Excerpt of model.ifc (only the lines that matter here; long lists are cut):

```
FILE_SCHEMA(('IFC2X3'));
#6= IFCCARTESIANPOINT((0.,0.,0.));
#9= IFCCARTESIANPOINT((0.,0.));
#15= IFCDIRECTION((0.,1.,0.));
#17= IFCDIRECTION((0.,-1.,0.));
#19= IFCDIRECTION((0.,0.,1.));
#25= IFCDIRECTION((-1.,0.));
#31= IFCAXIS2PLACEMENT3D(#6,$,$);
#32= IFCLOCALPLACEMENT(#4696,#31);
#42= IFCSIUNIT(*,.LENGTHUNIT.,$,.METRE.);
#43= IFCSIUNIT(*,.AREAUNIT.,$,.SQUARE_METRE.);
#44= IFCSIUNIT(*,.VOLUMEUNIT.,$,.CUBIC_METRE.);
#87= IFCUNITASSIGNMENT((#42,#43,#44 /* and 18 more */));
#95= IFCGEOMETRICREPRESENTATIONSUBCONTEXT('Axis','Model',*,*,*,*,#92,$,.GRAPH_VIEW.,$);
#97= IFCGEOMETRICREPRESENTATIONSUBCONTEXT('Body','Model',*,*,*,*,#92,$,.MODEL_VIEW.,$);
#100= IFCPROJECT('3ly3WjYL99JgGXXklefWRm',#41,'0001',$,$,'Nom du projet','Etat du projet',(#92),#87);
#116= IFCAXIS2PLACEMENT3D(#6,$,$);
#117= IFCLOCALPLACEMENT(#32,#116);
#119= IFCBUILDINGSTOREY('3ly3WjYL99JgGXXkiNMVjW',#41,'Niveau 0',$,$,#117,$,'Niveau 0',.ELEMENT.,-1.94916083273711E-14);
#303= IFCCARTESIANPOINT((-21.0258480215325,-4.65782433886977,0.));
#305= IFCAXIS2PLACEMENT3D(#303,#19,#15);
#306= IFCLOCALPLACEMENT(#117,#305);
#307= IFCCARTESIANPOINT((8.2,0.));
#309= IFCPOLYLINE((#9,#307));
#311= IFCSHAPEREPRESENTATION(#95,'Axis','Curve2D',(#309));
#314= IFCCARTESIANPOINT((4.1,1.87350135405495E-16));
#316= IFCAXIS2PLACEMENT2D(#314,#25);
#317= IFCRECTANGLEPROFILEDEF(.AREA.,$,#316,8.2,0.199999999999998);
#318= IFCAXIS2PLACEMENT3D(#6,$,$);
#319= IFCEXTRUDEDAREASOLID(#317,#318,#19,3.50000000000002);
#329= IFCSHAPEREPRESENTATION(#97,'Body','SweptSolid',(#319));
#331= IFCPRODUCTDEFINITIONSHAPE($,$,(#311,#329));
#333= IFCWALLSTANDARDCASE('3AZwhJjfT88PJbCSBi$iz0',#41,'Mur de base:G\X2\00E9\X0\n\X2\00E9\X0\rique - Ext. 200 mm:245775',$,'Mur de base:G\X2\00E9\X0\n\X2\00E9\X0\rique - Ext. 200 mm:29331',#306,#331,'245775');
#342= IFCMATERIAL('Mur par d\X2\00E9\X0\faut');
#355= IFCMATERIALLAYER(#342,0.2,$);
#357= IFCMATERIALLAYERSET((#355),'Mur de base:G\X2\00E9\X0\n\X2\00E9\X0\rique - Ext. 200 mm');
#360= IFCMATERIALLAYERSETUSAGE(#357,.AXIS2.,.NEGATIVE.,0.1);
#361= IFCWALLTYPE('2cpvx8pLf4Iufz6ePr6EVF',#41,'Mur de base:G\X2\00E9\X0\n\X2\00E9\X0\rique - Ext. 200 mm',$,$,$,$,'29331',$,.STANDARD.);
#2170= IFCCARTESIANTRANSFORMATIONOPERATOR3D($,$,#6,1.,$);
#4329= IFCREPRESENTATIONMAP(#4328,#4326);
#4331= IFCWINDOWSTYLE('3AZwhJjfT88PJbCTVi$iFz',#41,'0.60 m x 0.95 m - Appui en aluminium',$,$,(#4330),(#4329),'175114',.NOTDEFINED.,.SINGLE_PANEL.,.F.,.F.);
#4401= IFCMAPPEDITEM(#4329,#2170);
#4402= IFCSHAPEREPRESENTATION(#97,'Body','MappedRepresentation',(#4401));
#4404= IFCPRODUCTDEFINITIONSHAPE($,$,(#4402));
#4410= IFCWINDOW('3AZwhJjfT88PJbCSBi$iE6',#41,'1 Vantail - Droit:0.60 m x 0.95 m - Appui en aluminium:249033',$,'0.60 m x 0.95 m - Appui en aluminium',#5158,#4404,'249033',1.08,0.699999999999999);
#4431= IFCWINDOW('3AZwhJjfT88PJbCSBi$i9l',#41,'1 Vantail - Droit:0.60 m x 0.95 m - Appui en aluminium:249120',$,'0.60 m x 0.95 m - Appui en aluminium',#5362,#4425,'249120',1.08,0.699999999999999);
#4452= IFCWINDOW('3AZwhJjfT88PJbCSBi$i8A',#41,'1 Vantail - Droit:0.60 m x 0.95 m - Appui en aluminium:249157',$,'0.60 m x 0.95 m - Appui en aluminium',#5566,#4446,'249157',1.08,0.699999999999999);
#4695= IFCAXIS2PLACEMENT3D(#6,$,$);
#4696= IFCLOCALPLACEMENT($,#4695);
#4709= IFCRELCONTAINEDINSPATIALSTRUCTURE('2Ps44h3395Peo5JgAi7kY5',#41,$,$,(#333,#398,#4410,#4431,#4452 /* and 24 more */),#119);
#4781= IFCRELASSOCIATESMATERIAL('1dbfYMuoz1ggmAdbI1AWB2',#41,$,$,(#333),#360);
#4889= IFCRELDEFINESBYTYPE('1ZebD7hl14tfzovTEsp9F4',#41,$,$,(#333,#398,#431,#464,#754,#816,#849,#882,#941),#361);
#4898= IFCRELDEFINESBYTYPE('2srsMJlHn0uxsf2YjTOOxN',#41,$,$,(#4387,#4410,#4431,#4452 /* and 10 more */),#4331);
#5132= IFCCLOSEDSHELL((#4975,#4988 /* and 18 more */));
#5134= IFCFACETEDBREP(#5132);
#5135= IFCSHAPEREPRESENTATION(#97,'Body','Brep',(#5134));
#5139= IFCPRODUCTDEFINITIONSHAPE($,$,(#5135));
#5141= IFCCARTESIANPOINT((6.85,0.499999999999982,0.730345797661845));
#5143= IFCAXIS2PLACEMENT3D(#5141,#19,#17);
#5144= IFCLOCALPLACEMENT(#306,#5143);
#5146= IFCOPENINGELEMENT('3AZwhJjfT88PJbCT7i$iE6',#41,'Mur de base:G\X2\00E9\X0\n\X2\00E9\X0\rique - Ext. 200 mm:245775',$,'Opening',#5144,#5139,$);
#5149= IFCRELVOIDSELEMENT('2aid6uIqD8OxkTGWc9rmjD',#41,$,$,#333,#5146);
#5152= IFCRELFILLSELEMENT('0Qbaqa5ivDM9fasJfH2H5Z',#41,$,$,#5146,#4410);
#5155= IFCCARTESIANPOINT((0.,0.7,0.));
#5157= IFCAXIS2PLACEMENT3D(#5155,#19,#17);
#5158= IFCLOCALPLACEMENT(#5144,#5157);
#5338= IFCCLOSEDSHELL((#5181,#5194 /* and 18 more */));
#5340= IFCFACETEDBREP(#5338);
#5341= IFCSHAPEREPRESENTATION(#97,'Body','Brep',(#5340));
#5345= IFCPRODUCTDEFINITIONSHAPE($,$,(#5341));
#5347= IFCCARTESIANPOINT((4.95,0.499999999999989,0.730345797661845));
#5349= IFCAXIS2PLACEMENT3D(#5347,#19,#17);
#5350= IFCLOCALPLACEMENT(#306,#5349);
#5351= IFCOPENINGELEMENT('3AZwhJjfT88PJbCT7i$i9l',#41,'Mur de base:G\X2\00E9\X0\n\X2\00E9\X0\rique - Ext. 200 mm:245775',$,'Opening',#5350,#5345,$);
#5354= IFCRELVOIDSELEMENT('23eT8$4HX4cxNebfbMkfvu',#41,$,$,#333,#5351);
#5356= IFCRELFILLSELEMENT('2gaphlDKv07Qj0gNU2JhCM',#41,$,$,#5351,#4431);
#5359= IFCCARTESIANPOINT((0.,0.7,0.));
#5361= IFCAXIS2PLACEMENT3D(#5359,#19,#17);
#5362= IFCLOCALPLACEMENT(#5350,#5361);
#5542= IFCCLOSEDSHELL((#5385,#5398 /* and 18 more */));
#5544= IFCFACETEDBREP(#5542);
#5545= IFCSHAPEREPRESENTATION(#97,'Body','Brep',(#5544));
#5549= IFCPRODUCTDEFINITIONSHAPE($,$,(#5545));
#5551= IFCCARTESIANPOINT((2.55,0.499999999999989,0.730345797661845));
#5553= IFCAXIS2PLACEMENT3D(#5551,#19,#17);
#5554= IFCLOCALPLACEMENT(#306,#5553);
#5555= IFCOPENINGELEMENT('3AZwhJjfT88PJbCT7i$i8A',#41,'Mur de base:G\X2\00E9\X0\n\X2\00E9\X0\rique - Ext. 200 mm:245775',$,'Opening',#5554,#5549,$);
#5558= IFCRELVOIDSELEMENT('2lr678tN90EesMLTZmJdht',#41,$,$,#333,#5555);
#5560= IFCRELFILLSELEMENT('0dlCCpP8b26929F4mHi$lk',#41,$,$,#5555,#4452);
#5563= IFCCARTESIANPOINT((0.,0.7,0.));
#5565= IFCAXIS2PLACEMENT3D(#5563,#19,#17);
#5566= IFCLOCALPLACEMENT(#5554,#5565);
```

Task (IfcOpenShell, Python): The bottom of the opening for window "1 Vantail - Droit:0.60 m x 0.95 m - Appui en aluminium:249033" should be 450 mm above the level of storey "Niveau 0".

```python
import numpy as np
import ifcopenshell
import ifcopenshell.api.geometry
import ifcopenshell.geom
import ifcopenshell.util.element
import ifcopenshell.util.placement
import ifcopenshell.util.shape
import ifcopenshell.util.unit

model = ifcopenshell.open("model.ifc")
unit_scale = ifcopenshell.util.unit.calculate_unit_scale(model)

window = model.by_guid("3AZwhJjfT88PJbCSBi$iE6")
opening = window.FillsVoids[0].RelatingOpeningElement
storey = ifcopenshell.util.element.get_container(window, ifc_class="IfcBuildingStorey")
level = ifcopenshell.util.placement.get_local_placement(storey.ObjectPlacement)[2, 3]

# The opening's origin need not be at the sill, so measure its lowest point.
shape = ifcopenshell.geom.create_shape(ifcopenshell.geom.settings(), opening)
bottom = ifcopenshell.util.shape.get_shape_bottom_elevation(shape, shape.geometry) / unit_scale
dz = level + 0.45 - bottom

shift = np.array([0.0, 0.0, dz])
# The window is placed relative to its opening, so it follows when the opening moves.
matrix = ifcopenshell.util.placement.get_local_placement(opening.ObjectPlacement)
matrix[:3, 3] += shift
ifcopenshell.api.geometry.edit_object_placement(
    model, product=opening, matrix=matrix, is_si=False, should_transform_children=True
)

print(f"moved by {dz * unit_scale:+.3f} m")

model.write("model_v2.ifc")
```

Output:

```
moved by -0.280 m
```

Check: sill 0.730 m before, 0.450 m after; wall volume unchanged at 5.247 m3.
